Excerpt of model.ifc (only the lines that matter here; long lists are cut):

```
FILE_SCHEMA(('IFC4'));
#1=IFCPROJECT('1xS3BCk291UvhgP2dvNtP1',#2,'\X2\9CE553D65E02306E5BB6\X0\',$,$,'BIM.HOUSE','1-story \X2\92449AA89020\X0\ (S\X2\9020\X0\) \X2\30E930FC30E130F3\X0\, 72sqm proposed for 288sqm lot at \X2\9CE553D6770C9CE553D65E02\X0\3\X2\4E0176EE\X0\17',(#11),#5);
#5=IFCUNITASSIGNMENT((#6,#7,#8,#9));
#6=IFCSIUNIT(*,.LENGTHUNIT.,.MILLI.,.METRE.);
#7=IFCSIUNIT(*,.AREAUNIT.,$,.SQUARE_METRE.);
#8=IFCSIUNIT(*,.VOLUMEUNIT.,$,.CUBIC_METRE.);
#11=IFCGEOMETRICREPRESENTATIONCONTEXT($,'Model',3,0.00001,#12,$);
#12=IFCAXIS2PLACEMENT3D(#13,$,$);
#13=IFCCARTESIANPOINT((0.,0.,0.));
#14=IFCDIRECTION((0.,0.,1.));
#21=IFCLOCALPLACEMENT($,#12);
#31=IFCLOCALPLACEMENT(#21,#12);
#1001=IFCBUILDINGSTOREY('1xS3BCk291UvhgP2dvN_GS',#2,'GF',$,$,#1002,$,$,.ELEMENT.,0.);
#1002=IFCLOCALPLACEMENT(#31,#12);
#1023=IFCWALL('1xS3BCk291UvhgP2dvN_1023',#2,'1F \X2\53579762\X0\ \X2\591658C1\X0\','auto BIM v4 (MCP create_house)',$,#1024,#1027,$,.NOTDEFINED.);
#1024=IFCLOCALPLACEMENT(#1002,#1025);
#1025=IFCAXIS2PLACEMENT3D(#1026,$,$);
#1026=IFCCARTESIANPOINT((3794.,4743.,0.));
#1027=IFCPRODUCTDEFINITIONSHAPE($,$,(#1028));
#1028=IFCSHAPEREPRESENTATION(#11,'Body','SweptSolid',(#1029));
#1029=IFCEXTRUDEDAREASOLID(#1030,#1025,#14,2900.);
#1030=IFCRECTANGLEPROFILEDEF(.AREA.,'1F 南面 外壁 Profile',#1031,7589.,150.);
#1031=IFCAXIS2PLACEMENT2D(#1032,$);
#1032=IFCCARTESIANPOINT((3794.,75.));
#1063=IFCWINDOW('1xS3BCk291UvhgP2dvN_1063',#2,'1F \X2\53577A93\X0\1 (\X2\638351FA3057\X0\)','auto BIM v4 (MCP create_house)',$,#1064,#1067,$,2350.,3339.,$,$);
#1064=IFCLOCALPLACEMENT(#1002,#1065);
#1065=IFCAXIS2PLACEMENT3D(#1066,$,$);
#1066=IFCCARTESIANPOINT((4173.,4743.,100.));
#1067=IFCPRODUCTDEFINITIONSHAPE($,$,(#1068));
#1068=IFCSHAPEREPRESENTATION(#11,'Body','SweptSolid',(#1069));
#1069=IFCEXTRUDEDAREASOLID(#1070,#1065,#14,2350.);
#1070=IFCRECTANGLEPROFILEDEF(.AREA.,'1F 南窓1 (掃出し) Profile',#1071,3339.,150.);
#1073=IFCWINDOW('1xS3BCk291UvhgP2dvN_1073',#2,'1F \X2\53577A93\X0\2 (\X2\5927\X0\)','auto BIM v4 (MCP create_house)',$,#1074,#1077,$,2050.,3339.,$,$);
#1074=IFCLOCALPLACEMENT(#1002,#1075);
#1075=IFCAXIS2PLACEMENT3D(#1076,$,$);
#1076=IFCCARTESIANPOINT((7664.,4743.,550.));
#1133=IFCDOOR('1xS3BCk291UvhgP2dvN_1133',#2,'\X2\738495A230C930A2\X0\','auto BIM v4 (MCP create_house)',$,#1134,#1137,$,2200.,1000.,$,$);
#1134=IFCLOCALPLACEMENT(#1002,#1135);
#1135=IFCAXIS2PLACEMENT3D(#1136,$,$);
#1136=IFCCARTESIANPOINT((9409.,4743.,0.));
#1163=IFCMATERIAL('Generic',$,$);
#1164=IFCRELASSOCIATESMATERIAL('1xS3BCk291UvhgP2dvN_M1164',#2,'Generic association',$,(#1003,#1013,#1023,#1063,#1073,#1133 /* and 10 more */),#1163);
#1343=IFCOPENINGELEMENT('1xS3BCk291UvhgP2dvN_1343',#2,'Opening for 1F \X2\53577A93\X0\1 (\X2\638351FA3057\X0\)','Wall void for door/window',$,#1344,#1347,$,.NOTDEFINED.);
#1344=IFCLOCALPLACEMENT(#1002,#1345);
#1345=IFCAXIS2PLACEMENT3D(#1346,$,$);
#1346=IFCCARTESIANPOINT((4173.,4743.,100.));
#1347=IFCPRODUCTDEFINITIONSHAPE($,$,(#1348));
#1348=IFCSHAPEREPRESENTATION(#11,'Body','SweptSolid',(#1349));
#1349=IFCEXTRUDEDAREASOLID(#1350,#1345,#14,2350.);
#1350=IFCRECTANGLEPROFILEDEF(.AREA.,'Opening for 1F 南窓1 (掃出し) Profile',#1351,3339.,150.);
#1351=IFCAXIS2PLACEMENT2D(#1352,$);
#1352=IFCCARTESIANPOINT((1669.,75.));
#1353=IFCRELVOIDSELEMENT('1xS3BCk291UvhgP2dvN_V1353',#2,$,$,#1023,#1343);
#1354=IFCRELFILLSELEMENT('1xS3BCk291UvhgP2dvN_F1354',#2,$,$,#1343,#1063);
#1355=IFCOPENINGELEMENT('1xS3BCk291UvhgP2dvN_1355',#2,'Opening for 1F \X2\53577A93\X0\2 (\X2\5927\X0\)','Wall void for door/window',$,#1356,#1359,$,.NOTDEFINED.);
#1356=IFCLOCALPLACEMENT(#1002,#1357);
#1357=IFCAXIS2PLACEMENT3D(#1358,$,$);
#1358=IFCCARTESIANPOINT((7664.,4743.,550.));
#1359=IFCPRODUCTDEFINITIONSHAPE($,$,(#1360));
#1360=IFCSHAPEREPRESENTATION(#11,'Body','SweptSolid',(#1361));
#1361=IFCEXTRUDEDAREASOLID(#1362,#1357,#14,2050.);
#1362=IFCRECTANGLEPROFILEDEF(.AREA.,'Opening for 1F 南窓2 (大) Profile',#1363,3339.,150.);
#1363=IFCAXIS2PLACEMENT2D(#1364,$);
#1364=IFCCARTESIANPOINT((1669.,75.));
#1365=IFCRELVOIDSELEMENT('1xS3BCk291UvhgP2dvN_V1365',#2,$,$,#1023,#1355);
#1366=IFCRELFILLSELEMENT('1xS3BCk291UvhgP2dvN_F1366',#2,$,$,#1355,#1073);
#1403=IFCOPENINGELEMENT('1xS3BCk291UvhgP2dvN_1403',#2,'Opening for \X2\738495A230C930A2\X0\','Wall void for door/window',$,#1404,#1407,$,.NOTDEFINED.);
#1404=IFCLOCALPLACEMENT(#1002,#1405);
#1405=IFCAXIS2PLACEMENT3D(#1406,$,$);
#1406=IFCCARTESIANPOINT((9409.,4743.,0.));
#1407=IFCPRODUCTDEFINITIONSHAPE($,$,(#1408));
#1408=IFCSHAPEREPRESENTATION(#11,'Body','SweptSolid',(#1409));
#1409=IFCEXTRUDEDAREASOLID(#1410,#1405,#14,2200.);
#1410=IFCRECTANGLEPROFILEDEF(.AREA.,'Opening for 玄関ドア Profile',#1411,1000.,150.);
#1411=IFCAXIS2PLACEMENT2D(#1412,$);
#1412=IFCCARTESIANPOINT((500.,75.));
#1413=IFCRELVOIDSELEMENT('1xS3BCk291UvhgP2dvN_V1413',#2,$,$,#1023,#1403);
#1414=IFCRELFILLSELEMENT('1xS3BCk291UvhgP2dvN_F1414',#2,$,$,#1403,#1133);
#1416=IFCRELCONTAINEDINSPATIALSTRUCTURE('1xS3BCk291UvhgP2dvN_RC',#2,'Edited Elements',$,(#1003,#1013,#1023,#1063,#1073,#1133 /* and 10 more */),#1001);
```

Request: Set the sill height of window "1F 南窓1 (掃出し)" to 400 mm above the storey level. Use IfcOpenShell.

```python
import numpy as np
import ifcopenshell
import ifcopenshell.api.geometry
import ifcopenshell.geom
import ifcopenshell.util.element
import ifcopenshell.util.placement
import ifcopenshell.util.shape
import ifcopenshell.util.unit

model = ifcopenshell.open("model.ifc")
unit_scale = ifcopenshell.util.unit.calculate_unit_scale(model)

window = model.by_guid("1xS3BCk291UvhgP2dvN_1063")
opening = window.FillsVoids[0].RelatingOpeningElement
storey = ifcopenshell.util.element.get_container(window, ifc_class="IfcBuildingStorey")
level = ifcopenshell.util.placement.get_local_placement(storey.ObjectPlacement)[2, 3]

# The opening's origin need not be at the sill, so measure its lowest point.
shape = ifcopenshell.geom.create_shape(ifcopenshell.geom.settings(), opening)
bottom = ifcopenshell.util.shape.get_shape_bottom_elevation(shape, shape.geometry) / unit_scale
dz = level + 0.4 / unit_scale - bottom

shift = np.array([0.0, 0.0, dz])
# The window is not placed relative to its opening, so move both.
for product in (opening, window):
    matrix = ifcopenshell.util.placement.get_local_placement(product.ObjectPlacement)
    matrix[:3, 3] += shift
    ifcopenshell.api.geometry.edit_object_placement(model, product=product, matrix=matrix, is_si=False)

print(f"moved by {dz * unit_scale:+.3f} m")

model.write("model_updated.ifc")
```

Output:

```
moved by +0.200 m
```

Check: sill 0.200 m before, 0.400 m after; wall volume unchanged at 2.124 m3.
